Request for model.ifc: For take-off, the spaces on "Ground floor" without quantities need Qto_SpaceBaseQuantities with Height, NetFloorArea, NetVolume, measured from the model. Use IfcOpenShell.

First a look at what the model holds.

```python
import ifcopenshell
import ifcopenshell.util.element
import ifcopenshell.util.unit

model = ifcopenshell.open("model.ifc")
print(model.schema)
for unit_type in ("LENGTHUNIT", "AREAUNIT", "VOLUMEUNIT"):
    print(unit_type, ifcopenshell.util.unit.calculate_unit_scale(model, unit_type))
storey = next(s for s in model.by_type("IfcBuildingStorey") if s.Name == "Ground floor")
spaces = [e for e in ifcopenshell.util.element.get_decomposition(storey) if e.is_a("IfcSpace")]
for e in sorted(spaces, key=lambda e: e.id()):
    print(e.id(), e.is_a(), e.Name, list(ifcopenshell.util.element.get_psets(e, qtos_only=True)), sep=" | ")
```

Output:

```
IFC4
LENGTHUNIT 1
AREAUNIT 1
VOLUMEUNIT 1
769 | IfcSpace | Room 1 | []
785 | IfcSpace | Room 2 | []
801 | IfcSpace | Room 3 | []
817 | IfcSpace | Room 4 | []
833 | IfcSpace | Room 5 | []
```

```python
import ifcopenshell
import ifcopenshell.api.pset
import ifcopenshell.geom
import ifcopenshell.util.element
import ifcopenshell.util.shape
import ifcopenshell.util.unit

model = ifcopenshell.open("model.ifc")
unit_scale = ifcopenshell.util.unit.calculate_unit_scale(model)
area_scale = ifcopenshell.util.unit.calculate_unit_scale(model, "AREAUNIT")
volume_scale = ifcopenshell.util.unit.calculate_unit_scale(model, "VOLUMEUNIT")
settings = ifcopenshell.geom.settings()

storey = next(s for s in model.by_type("IfcBuildingStorey") if s.Name == "Ground floor")
spaces = [e for e in ifcopenshell.util.element.get_decomposition(storey) if e.is_a("IfcSpace")]

for e in sorted(spaces, key=lambda e: e.id()):
    if ifcopenshell.util.element.get_psets(e, qtos_only=True, should_inherit=False):
        continue
    # Geometry comes back in metres, in the element's own axes.
    shape = ifcopenshell.geom.create_shape(settings, e)
    values = {
        "Height": ifcopenshell.util.shape.get_z(shape.geometry) / unit_scale,
        "NetFloorArea": ifcopenshell.util.shape.get_footprint_area(shape.geometry) / area_scale,
        "NetVolume": ifcopenshell.util.shape.get_volume(shape.geometry) / volume_scale,
    }
    qto = ifcopenshell.api.pset.add_qto(model, product=e, name="Qto_SpaceBaseQuantities")
    ifcopenshell.api.pset.edit_qto(model, qto=qto, properties=values)
    print(e.id(), {k: round(v, 3) for k, v in values.items()})

model.write("model_v2.ifc")
```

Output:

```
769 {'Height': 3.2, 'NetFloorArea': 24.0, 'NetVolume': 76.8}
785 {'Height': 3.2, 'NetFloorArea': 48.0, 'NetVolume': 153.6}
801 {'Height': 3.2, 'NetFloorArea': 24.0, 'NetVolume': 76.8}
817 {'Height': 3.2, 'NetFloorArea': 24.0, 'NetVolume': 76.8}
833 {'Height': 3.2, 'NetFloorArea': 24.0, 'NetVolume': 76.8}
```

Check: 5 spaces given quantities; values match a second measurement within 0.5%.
